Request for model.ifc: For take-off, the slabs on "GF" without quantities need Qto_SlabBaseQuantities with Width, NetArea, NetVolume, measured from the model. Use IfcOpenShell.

First a look at what the model holds.

```python
import ifcopenshell
import ifcopenshell.util.element
import ifcopenshell.util.unit

model = ifcopenshell.open("model.ifc")
print(model.schema)
for unit_type in ("LENGTHUNIT", "AREAUNIT", "VOLUMEUNIT"):
    print(unit_type, ifcopenshell.util.unit.calculate_unit_scale(model, unit_type))
storey = next(s for s in model.by_type("IfcBuildingStorey") if s.Name == "GF")
slabs = [e for e in ifcopenshell.util.element.get_decomposition(storey) if e.is_a("IfcSlab")]
for e in sorted(slabs, key=lambda e: e.id()):
    print(e.id(), e.is_a(), e.Name, list(ifcopenshell.util.element.get_psets(e, qtos_only=True)), sep=" | ")
```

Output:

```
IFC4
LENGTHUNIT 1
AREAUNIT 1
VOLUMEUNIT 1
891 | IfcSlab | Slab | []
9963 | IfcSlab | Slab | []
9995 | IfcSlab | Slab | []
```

```python
import ifcopenshell
import ifcopenshell.api.pset
import ifcopenshell.geom
import ifcopenshell.util.element
import ifcopenshell.util.shape
import ifcopenshell.util.unit

model = ifcopenshell.open("model.ifc")
unit_scale = ifcopenshell.util.unit.calculate_unit_scale(model)
area_scale = ifcopenshell.util.unit.calculate_unit_scale(model, "AREAUNIT")
volume_scale = ifcopenshell.util.unit.calculate_unit_scale(model, "VOLUMEUNIT")
settings = ifcopenshell.geom.settings()

storey = next(s for s in model.by_type("IfcBuildingStorey") if s.Name == "GF")
slabs = [e for e in ifcopenshell.util.element.get_decomposition(storey) if e.is_a("IfcSlab")]

for e in sorted(slabs, key=lambda e: e.id()):
    if ifcopenshell.util.element.get_psets(e, qtos_only=True, should_inherit=False):
        continue
    # Geometry comes back in metres, in the element's own axes.
    shape = ifcopenshell.geom.create_shape(settings, e)
    values = {
        "Width": ifcopenshell.util.shape.get_z(shape.geometry) / unit_scale,
        "NetArea": ifcopenshell.util.shape.get_footprint_area(shape.geometry) / area_scale,
        "NetVolume": ifcopenshell.util.shape.get_volume(shape.geometry) / volume_scale,
    }
    qto = ifcopenshell.api.pset.add_qto(model, product=e, name="Qto_SlabBaseQuantities")
    ifcopenshell.api.pset.edit_qto(model, qto=qto, properties=values)
    print(e.id(), {k: round(v, 3) for k, v in values.items()})

model.write("model_updated.ifc")
```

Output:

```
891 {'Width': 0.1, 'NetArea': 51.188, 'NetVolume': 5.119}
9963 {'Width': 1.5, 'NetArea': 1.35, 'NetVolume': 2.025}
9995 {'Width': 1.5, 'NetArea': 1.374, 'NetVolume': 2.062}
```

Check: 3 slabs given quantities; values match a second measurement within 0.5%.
